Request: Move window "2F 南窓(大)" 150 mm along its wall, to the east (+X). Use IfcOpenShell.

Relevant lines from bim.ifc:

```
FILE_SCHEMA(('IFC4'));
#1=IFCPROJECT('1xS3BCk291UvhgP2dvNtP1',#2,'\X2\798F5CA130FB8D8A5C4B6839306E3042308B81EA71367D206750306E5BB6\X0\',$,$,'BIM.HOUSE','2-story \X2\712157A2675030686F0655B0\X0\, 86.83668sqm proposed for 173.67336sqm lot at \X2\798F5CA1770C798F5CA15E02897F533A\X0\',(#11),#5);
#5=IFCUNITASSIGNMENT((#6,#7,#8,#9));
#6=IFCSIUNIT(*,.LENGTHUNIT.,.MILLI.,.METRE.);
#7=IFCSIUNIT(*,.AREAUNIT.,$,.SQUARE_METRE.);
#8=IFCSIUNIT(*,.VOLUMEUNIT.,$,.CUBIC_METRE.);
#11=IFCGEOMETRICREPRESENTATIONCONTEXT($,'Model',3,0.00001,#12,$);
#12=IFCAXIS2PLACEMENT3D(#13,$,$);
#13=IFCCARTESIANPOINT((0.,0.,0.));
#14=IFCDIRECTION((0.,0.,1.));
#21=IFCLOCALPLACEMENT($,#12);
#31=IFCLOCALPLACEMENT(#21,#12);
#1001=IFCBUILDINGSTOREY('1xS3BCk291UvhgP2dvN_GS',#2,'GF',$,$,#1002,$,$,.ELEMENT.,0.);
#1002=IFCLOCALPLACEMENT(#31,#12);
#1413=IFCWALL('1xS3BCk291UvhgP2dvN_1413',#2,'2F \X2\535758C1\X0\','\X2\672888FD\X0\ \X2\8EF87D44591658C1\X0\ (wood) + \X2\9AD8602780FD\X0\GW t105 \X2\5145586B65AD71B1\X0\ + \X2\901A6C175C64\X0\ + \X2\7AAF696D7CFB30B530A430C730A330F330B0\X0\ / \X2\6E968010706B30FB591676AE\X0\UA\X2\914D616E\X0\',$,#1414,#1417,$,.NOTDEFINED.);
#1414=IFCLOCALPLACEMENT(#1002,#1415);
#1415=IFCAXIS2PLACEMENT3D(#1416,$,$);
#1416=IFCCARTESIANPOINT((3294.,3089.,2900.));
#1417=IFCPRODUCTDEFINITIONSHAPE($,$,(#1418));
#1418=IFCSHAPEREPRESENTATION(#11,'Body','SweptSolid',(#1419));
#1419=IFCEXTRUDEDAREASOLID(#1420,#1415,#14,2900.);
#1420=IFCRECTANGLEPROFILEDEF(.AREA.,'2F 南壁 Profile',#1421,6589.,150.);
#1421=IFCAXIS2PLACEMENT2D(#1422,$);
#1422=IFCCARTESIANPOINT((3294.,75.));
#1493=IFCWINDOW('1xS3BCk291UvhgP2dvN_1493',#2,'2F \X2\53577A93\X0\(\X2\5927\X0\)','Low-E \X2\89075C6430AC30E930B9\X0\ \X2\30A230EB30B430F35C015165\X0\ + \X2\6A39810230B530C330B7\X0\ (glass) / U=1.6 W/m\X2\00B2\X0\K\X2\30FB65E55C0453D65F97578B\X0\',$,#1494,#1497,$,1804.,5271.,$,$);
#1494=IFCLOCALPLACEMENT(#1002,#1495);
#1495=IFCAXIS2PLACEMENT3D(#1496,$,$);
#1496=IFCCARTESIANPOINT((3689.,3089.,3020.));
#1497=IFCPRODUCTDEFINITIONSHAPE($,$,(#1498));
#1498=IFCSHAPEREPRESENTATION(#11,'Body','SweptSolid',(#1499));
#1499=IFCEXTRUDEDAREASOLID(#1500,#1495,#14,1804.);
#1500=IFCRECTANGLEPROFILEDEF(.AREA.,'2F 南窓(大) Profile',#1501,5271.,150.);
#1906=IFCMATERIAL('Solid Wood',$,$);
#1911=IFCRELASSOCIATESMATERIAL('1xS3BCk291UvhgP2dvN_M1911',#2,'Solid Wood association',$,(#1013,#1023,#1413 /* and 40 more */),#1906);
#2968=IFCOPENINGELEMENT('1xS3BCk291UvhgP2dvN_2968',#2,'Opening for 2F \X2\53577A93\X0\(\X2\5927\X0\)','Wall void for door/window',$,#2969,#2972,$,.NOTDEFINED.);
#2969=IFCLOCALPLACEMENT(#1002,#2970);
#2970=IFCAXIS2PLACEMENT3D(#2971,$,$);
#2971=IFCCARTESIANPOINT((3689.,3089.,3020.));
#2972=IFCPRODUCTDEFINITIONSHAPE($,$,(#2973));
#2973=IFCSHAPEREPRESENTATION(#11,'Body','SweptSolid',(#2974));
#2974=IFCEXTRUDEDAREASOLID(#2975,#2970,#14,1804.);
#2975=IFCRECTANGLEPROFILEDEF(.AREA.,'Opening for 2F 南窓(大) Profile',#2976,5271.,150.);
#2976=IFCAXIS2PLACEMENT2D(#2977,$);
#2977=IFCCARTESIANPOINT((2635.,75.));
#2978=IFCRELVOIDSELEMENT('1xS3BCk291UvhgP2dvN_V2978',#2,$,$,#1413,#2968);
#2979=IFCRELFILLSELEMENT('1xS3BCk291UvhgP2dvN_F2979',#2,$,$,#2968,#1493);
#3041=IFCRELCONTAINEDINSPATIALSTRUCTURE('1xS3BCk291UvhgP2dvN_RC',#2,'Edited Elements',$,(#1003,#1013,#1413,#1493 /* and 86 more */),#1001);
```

```python
import ifcopenshell
import ifcopenshell.api.geometry
import ifcopenshell.util.placement
import ifcopenshell.util.unit

model = ifcopenshell.open("bim.ifc")
unit_scale = ifcopenshell.util.unit.calculate_unit_scale(model)

window = model.by_guid("1xS3BCk291UvhgP2dvN_1493")
opening = window.FillsVoids[0].RelatingOpeningElement
wall = opening.VoidsElements[0].RelatingBuildingElement

wall_matrix = ifcopenshell.util.placement.get_local_placement(wall.ObjectPlacement)
shift = wall_matrix[:3, 0] * 0.15 / unit_scale
before = ifcopenshell.util.placement.get_local_placement(window.ObjectPlacement)[:3, 3].copy()

# The window is not placed relative to its opening, so move both.
for product in (opening, window):
    matrix = ifcopenshell.util.placement.get_local_placement(product.ObjectPlacement)
    matrix[:3, 3] += shift
    ifcopenshell.api.geometry.edit_object_placement(model, product=product, matrix=matrix, is_si=False)

after = ifcopenshell.util.placement.get_local_placement(window.ObjectPlacement)[:3, 3]
print("window moved by", (after - before).round(3) + 0.0)

model.write("bim_v2.ifc")
```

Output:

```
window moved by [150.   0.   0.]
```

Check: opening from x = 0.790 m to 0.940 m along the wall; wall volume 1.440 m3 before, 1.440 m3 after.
